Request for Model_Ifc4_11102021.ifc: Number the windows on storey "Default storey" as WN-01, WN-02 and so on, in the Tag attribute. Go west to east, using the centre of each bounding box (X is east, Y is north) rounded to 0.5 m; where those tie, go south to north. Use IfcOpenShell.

First a look at what the model holds.

```python
import ifcopenshell
import ifcopenshell.util.element
import ifcopenshell.util.placement

model = ifcopenshell.open("Model_Ifc4_11102021.ifc")
print(model.schema)
storey = next(s for s in model.by_type("IfcBuildingStorey") if s.Name == "Default storey")
windows = [e for e in ifcopenshell.util.element.get_decomposition(storey) if e.is_a("IfcWindow")]
for e in sorted(windows, key=lambda e: e.id()):
    origin = ifcopenshell.util.placement.get_local_placement(e.ObjectPlacement)[:3, 3]
    print(e.id(), e.Tag, e.Name, origin.round(2) + 0.0, sep=" | ")
```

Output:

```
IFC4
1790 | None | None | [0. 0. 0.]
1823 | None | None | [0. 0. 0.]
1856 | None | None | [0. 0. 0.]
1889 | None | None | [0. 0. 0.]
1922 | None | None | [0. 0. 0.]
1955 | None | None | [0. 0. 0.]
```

```python
import ifcopenshell
import ifcopenshell.geom
import ifcopenshell.util.element
import ifcopenshell.util.shape

model = ifcopenshell.open("Model_Ifc4_11102021.ifc")
settings = ifcopenshell.geom.settings()
settings.set("use-world-coords", True)


def centre(element):
    shape = ifcopenshell.geom.create_shape(settings, element)
    return ifcopenshell.util.shape.get_bbox_centroid(shape.geometry)


storey = next(s for s in model.by_type("IfcBuildingStorey") if s.Name == "Default storey")
windows = [e for e in ifcopenshell.util.element.get_decomposition(storey) if e.is_a("IfcWindow")]

# Insertion points can sit at a corner or the storey origin, so sort by the geometry (in metres).
centres = {e: centre(e) for e in windows}
windows.sort(key=lambda e: (round(centres[e][0] / 0.5), centres[e][1]))

for i, e in enumerate(windows, start=1):
    number = f"WN-{i:02d}"
    e.Tag = number
    print(e.id(), number)

model.write("Model_Ifc4_11102021_edited.ifc")
```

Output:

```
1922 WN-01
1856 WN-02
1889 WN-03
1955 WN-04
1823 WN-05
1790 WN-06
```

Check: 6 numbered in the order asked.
